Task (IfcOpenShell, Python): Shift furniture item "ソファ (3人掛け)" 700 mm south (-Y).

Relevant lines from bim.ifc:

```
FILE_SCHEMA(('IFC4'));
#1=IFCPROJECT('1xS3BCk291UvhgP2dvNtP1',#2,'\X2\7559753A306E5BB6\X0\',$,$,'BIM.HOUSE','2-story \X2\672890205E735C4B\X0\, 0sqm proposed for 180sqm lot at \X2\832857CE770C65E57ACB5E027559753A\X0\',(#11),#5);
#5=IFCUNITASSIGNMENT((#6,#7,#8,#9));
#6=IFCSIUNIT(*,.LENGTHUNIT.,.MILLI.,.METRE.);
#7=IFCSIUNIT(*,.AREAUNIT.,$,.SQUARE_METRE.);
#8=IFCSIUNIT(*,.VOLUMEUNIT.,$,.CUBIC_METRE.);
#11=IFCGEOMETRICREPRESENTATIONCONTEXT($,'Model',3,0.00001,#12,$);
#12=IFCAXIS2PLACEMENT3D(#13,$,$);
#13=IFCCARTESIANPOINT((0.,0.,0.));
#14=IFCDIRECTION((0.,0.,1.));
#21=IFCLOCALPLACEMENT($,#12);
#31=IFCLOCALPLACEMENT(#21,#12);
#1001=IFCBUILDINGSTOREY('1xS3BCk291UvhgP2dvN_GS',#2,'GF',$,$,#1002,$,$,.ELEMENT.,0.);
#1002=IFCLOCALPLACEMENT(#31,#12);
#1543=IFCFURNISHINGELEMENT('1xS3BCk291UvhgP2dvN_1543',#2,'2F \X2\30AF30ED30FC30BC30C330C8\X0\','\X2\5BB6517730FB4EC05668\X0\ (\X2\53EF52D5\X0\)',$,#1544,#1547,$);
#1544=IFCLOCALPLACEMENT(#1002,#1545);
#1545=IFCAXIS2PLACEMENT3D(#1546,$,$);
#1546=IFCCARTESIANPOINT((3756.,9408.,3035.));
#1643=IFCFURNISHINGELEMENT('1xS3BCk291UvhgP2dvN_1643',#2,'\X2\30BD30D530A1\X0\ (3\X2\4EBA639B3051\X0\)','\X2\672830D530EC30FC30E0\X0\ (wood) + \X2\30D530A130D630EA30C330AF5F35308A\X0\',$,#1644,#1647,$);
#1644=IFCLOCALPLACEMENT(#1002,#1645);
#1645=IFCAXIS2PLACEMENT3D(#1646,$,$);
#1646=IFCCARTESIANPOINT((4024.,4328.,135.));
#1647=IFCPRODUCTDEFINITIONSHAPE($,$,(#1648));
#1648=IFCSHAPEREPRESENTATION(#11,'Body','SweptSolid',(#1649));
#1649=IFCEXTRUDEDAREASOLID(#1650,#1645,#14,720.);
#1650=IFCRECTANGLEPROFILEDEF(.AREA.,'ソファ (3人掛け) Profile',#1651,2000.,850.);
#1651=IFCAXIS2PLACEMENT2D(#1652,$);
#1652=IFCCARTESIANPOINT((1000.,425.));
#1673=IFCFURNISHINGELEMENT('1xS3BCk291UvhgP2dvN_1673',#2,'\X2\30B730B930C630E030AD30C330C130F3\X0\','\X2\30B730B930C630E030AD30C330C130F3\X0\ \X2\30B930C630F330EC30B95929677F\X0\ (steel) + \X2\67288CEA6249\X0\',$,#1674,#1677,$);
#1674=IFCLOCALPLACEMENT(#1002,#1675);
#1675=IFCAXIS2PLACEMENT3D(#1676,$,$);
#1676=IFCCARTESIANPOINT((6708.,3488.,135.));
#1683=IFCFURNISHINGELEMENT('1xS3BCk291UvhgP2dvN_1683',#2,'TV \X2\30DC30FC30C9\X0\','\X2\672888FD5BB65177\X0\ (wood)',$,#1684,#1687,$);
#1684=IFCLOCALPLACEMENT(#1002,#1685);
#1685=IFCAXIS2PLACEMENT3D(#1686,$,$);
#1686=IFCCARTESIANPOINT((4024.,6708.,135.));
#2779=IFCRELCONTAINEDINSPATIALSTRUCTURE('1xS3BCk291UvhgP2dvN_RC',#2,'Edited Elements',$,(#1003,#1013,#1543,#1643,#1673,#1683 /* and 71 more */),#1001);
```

```python
import ifcopenshell
import ifcopenshell.api.geometry
import ifcopenshell.util.placement

model = ifcopenshell.open("bim.ifc")

item = model.by_guid("1xS3BCk291UvhgP2dvN_1643")
matrix = ifcopenshell.util.placement.get_local_placement(item.ObjectPlacement)
matrix[1, 3] -= 700.0
ifcopenshell.api.geometry.edit_object_placement(model, product=item, matrix=matrix, is_si=False)

print(ifcopenshell.util.placement.get_local_placement(item.ObjectPlacement).round(3) + 0.0)

model.write("bim_updated.ifc")
```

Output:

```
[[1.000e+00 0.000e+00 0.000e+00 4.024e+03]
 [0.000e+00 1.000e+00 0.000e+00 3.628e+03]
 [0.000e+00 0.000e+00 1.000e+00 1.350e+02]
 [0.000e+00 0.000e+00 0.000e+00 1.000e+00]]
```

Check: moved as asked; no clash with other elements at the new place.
